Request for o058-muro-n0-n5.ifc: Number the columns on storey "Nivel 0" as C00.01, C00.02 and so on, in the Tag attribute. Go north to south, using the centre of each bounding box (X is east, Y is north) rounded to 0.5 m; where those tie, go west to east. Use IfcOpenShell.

First a look at what the model holds.

```python
import ifcopenshell
import ifcopenshell.util.element
import ifcopenshell.util.placement

model = ifcopenshell.open("o058-muro-n0-n5.ifc")
print(model.schema)
storey = next(s for s in model.by_type("IfcBuildingStorey") if s.Name == "Nivel 0")
columns = [e for e in ifcopenshell.util.element.get_decomposition(storey) if e.is_a("IfcColumn")]
for e in sorted(columns, key=lambda e: e.id()):
    origin = ifcopenshell.util.placement.get_local_placement(e.ObjectPlacement)[:3, 3]
    print(e.id(), e.Tag, e.Name, origin.round(2) + 0.0, sep=" | ")
```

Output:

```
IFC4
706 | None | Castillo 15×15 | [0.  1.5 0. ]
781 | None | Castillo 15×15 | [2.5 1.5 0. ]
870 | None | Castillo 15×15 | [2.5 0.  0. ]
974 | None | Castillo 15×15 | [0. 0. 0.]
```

```python
import ifcopenshell
import ifcopenshell.geom
import ifcopenshell.util.element
import ifcopenshell.util.shape

model = ifcopenshell.open("o058-muro-n0-n5.ifc")
settings = ifcopenshell.geom.settings()
settings.set("use-world-coords", True)


def centre(element):
    shape = ifcopenshell.geom.create_shape(settings, element)
    return ifcopenshell.util.shape.get_bbox_centroid(shape.geometry)


storey = next(s for s in model.by_type("IfcBuildingStorey") if s.Name == "Nivel 0")
columns = [e for e in ifcopenshell.util.element.get_decomposition(storey) if e.is_a("IfcColumn")]

# Insertion points can sit at a corner or the storey origin, so sort by the geometry (in metres).
centres = {e: centre(e) for e in columns}
columns.sort(key=lambda e: (-round(centres[e][1] / 0.5), centres[e][0]))

for i, e in enumerate(columns, start=1):
    number = f"C00.{i:02d}"
    e.Tag = number
    print(e.id(), number)

model.write("o058-muro-n0-n5-out.ifc")
```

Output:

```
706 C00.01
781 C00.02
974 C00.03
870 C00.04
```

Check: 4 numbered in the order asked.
